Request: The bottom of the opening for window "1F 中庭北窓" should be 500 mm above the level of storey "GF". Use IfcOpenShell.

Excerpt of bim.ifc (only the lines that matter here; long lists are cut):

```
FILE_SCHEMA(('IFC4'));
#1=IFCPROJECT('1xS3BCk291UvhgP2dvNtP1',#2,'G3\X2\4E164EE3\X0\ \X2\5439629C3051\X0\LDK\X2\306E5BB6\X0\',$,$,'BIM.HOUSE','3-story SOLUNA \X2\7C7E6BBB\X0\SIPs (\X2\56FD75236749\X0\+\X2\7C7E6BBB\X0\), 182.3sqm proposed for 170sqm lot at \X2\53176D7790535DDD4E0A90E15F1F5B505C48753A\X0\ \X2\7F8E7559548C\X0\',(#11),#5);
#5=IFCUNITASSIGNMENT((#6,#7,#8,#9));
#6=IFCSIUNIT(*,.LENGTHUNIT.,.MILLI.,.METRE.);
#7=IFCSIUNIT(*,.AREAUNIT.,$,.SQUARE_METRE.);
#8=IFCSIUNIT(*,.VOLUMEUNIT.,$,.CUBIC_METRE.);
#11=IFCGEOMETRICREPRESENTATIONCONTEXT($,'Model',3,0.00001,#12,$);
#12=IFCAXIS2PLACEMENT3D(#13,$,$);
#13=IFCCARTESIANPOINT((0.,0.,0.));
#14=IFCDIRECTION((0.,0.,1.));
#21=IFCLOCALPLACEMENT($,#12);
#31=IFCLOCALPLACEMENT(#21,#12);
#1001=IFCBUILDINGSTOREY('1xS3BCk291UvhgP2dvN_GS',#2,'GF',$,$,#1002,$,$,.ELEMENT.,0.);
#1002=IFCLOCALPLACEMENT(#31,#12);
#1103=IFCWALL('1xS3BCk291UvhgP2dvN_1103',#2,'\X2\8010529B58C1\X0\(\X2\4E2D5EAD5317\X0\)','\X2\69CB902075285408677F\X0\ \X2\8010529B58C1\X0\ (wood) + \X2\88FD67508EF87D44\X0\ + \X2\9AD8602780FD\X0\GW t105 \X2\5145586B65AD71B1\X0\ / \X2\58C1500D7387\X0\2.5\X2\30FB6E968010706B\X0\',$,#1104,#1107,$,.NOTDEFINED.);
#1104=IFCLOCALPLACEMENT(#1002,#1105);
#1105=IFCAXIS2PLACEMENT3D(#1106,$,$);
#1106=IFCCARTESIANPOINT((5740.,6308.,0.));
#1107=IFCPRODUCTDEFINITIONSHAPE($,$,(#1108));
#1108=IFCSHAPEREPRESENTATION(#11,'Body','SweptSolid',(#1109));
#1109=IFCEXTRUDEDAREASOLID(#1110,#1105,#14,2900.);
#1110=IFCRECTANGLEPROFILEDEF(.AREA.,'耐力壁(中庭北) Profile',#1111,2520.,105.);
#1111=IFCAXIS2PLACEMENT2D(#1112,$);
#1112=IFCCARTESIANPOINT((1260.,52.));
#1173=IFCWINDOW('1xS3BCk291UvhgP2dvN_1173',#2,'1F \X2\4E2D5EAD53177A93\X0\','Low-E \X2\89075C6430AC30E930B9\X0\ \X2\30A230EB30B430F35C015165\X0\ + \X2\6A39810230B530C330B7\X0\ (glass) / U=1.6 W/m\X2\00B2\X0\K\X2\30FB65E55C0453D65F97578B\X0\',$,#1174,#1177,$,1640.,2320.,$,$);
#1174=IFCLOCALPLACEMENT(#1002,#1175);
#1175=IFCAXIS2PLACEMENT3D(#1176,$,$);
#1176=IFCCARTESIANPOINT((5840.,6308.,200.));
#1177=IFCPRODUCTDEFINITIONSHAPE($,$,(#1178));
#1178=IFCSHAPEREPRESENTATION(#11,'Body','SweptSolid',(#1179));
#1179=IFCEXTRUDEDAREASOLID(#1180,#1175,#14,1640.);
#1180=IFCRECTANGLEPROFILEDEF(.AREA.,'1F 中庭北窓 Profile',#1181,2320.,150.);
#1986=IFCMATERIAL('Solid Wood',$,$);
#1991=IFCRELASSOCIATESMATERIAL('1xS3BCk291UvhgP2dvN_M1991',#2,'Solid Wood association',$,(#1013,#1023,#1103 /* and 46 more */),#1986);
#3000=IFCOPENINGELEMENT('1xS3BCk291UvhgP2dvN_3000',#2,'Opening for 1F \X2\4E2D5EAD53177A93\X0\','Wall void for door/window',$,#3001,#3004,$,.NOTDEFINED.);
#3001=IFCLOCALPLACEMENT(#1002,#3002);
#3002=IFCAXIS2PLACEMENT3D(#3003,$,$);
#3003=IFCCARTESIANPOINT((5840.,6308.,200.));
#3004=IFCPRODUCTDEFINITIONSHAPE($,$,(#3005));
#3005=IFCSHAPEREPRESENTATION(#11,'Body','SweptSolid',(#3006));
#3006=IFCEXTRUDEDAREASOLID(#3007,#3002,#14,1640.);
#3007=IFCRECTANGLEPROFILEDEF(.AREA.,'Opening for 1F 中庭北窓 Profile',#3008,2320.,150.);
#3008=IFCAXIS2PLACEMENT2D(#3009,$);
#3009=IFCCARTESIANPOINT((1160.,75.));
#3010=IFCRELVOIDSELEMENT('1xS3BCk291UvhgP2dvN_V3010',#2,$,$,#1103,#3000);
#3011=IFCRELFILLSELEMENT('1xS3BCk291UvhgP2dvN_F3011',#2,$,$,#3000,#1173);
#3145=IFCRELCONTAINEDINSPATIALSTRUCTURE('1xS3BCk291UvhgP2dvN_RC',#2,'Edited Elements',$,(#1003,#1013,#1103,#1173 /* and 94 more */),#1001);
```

```python
import numpy as np
import ifcopenshell
import ifcopenshell.api.geometry
import ifcopenshell.geom
import ifcopenshell.util.element
import ifcopenshell.util.placement
import ifcopenshell.util.shape
import ifcopenshell.util.unit

model = ifcopenshell.open("bim.ifc")
unit_scale = ifcopenshell.util.unit.calculate_unit_scale(model)

window = model.by_id(1173)
opening = window.FillsVoids[0].RelatingOpeningElement
storey = ifcopenshell.util.element.get_container(window, ifc_class="IfcBuildingStorey")
level = ifcopenshell.util.placement.get_local_placement(storey.ObjectPlacement)[2, 3]

# The opening's origin need not be at the sill, so measure its lowest point.
shape = ifcopenshell.geom.create_shape(ifcopenshell.geom.settings(), opening)
bottom = ifcopenshell.util.shape.get_shape_bottom_elevation(shape, shape.geometry) / unit_scale
dz = level + 0.5 / unit_scale - bottom

shift = np.array([0.0, 0.0, dz])
# The window is not placed relative to its opening, so move both.
for product in (opening, window):
    matrix = ifcopenshell.util.placement.get_local_placement(product.ObjectPlacement)
    matrix[:3, 3] += shift
    ifcopenshell.api.geometry.edit_object_placement(model, product=product, matrix=matrix, is_si=False)

print(f"moved by {dz * unit_scale:+.3f} m")

model.write("bim_updated.ifc")
```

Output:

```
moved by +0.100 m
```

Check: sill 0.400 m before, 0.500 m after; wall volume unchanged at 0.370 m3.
